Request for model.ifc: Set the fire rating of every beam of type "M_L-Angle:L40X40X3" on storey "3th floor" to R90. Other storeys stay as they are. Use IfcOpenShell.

First a look at what the model holds.

```python
import ifcopenshell
import ifcopenshell.util.element

model = ifcopenshell.open("model.ifc")
print(model.schema)
storey = next(s for s in model.by_type("IfcBuildingStorey") if s.Name == "3th floor")
beams = [e for e in ifcopenshell.util.element.get_decomposition(storey) if e.is_a("IfcBeam")]
seen = {}
for e in beams:
    element_type = ifcopenshell.util.element.get_type(e)
    key = (element_type.Name if element_type != e and element_type else None, ifcopenshell.util.element.get_pset(e, "Pset_BeamCommon", "FireRating"))
    seen[key] = seen.get(key, 0) + 1
for (name, value), count in sorted(seen.items(), key=str):
    print(count, "x", name, "|", value)
```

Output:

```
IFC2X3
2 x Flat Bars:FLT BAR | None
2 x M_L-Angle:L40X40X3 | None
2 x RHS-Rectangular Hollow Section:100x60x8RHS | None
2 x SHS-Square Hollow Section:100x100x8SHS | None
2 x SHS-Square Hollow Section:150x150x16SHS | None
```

```python
import ifcopenshell
import ifcopenshell.api.pset
import ifcopenshell.util.element

model = ifcopenshell.open("model.ifc")

storey = next(s for s in model.by_type("IfcBuildingStorey") if s.Name == "3th floor")
beams = [e for e in ifcopenshell.util.element.get_decomposition(storey) if e.is_a("IfcBeam")]

count = 0
for e in beams:
    element_type = ifcopenshell.util.element.get_type(e)
    if element_type in (None, e) or element_type.Name != "M_L-Angle:L40X40X3":
        continue
    # add_pset returns the element's existing set when there is one.
    pset = ifcopenshell.api.pset.add_pset(model, product=e, name="Pset_BeamCommon")
    ifcopenshell.api.pset.edit_pset(model, pset=pset, properties={"FireRating": "R90"})
    count += 1

print(count, "beams updated")

model.write("model-out.ifc")
```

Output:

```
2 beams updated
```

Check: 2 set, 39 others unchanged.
